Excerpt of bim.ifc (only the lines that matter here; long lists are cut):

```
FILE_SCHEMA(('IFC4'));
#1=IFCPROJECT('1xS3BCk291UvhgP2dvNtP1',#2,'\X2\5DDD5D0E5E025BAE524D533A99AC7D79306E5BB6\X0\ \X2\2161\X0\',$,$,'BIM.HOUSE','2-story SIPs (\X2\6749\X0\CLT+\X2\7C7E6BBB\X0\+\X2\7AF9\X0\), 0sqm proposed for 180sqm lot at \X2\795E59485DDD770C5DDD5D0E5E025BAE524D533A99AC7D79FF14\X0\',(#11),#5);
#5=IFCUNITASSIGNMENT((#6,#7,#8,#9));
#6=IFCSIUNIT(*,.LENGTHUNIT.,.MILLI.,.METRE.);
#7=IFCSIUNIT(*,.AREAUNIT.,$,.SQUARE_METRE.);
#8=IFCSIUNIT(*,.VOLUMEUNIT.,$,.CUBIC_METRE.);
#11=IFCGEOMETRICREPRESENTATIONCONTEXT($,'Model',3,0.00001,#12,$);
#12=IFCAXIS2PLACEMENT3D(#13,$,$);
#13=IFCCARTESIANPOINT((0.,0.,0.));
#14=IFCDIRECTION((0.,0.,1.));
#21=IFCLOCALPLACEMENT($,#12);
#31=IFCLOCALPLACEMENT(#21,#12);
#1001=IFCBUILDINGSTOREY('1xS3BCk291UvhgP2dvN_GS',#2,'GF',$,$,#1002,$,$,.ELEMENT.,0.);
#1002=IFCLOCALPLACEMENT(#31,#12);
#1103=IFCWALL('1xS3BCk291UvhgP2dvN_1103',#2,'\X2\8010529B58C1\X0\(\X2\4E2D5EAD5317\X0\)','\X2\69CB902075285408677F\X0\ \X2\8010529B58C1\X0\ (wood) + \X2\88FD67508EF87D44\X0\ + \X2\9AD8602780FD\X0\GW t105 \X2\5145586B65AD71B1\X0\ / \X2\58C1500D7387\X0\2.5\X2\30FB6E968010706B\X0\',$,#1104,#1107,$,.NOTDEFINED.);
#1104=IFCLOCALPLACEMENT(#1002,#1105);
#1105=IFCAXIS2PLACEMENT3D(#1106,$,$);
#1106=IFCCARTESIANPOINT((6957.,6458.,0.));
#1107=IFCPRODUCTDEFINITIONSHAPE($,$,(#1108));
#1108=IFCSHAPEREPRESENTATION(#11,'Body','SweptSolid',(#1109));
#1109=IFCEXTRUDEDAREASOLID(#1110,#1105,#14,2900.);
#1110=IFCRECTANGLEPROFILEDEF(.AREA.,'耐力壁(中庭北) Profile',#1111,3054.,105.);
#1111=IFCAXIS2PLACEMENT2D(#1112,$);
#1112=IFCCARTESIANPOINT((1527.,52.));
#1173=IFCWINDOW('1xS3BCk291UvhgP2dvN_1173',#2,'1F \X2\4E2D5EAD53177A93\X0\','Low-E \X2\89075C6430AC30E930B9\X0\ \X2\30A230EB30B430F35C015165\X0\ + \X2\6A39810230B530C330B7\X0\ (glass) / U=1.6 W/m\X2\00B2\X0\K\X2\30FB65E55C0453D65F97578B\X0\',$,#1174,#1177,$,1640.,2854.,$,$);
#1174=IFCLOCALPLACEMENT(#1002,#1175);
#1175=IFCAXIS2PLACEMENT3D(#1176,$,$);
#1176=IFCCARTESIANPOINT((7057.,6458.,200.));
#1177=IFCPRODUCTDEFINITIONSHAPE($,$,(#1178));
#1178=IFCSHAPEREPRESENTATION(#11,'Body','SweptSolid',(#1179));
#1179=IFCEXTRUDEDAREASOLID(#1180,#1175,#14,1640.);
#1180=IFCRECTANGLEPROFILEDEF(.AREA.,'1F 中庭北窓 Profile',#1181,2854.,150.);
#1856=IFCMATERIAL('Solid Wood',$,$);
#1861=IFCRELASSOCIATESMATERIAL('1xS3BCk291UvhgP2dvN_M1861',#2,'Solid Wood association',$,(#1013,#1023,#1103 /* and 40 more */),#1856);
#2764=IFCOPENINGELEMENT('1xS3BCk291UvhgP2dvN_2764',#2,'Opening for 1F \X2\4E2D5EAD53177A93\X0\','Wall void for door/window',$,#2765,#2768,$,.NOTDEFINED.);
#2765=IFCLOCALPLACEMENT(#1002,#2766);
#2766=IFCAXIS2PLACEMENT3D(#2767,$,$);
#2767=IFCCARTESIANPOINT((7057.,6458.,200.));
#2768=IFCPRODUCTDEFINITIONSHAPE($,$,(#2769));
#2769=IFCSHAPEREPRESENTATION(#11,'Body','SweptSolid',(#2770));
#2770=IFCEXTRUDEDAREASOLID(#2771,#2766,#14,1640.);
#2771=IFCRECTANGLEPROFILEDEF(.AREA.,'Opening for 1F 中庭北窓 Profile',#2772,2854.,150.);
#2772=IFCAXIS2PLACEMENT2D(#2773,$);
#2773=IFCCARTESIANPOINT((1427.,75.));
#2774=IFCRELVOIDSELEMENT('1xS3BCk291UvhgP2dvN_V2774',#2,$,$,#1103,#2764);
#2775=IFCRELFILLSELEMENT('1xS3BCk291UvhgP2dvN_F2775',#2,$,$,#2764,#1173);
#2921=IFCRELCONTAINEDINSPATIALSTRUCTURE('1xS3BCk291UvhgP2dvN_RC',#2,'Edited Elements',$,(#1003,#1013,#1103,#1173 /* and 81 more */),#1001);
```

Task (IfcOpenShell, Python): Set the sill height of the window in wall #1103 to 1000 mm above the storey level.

```python
import numpy as np
import ifcopenshell
import ifcopenshell.api.geometry
import ifcopenshell.geom
import ifcopenshell.util.element
import ifcopenshell.util.placement
import ifcopenshell.util.shape
import ifcopenshell.util.unit

model = ifcopenshell.open("bim.ifc")
unit_scale = ifcopenshell.util.unit.calculate_unit_scale(model)

window = model.by_guid("1xS3BCk291UvhgP2dvN_1173")
opening = window.FillsVoids[0].RelatingOpeningElement
storey = ifcopenshell.util.element.get_container(window, ifc_class="IfcBuildingStorey")
level = ifcopenshell.util.placement.get_local_placement(storey.ObjectPlacement)[2, 3]

# The opening's origin need not be at the sill, so measure its lowest point.
shape = ifcopenshell.geom.create_shape(ifcopenshell.geom.settings(), opening)
bottom = ifcopenshell.util.shape.get_shape_bottom_elevation(shape, shape.geometry) / unit_scale
dz = level + 1000.0 - bottom

shift = np.array([0.0, 0.0, dz])
# The window is not placed relative to its opening, so move both.
for product in (opening, window):
    matrix = ifcopenshell.util.placement.get_local_placement(product.ObjectPlacement)
    matrix[:3, 3] += shift
    ifcopenshell.api.geometry.edit_object_placement(model, product=product, matrix=matrix, is_si=False)

print(f"moved by {dz * unit_scale:+.3f} m")

model.write("bim-out.ifc")
```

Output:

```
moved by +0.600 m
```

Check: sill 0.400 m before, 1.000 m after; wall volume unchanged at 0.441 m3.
